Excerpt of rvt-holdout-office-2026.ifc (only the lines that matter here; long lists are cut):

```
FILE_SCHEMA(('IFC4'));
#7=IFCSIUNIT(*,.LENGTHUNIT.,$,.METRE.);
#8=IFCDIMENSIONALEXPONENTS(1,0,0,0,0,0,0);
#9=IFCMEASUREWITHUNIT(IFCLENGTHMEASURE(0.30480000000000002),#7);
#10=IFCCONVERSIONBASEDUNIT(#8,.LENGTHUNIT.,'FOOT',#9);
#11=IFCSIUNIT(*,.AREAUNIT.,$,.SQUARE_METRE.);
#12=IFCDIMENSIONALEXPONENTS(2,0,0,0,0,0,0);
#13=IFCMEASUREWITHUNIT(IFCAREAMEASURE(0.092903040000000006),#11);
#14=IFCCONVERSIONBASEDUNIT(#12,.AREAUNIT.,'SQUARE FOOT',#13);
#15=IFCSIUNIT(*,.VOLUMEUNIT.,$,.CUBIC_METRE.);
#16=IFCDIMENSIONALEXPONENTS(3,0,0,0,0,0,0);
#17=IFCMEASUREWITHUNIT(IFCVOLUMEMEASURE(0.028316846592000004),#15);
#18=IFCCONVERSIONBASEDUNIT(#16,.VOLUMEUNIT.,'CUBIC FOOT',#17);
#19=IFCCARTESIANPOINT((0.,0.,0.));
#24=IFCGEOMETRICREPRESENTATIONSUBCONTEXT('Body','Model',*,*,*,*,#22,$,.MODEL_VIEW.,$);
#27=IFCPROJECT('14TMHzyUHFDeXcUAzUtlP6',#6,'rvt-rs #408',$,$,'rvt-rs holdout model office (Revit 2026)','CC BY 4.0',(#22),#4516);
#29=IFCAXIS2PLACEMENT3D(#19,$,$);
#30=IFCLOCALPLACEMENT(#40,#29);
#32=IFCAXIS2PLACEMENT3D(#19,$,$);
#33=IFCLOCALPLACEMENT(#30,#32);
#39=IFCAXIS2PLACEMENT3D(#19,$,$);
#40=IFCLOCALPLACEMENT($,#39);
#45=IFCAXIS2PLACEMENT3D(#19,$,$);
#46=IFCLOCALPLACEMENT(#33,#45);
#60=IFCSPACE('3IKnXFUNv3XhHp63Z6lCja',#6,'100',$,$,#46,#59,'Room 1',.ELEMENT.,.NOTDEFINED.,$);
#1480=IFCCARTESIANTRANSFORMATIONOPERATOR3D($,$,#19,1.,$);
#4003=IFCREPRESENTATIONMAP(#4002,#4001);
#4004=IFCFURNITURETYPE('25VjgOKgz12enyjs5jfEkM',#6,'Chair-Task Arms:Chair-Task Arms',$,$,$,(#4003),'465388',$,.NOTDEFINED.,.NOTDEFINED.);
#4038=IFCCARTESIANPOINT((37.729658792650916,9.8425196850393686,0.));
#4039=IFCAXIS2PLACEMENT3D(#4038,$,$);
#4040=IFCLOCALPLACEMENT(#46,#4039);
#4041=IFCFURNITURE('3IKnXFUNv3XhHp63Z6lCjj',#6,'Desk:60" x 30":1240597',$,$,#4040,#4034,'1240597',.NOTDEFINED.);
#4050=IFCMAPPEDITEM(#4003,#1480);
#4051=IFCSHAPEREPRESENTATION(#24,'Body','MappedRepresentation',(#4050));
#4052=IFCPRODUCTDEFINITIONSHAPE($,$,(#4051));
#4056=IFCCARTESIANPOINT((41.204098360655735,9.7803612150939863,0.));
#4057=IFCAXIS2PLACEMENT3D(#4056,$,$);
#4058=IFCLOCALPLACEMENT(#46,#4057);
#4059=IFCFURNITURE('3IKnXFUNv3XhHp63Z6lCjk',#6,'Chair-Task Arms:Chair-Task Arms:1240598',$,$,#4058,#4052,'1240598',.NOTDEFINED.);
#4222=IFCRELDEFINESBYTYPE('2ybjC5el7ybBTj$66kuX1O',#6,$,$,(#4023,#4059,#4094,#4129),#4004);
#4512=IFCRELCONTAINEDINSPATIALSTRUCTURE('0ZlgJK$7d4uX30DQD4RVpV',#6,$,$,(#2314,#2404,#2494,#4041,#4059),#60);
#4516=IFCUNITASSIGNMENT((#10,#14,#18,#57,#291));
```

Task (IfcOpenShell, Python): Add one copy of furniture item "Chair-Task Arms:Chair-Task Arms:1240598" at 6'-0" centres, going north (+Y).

```python
import numpy as np
import ifcopenshell
import ifcopenshell.api.geometry
import ifcopenshell.api.root
import ifcopenshell.util.element
import ifcopenshell.util.placement
import ifcopenshell.util.unit

model = ifcopenshell.open("rvt-holdout-office-2026.ifc")
unit_scale = ifcopenshell.util.unit.calculate_unit_scale(model)


def reuse_history(source, copy):
    """copy_class also copies each property set's owner history, people and application; keep the originals."""
    for rel in copy.IsDefinedBy:
        if rel.is_a("IfcRelDefinesByProperties") and (history := rel.RelatingPropertyDefinition.OwnerHistory):
            rel.RelatingPropertyDefinition.OwnerHistory = source.OwnerHistory
            ifcopenshell.util.element.remove_deep2(model, history)


source = model.by_guid("3IKnXFUNv3XhHp63Z6lCjk")
base = ifcopenshell.util.placement.get_local_placement(source.ObjectPlacement)
step = np.array([0.0, 1.0, 0.0]) * 72 * 0.0254 / unit_scale

for i in range(1, 2):
    copy = ifcopenshell.api.root.copy_class(model, product=source)
    copy.Representation = ifcopenshell.util.element.copy_deep(
        model, source.Representation, exclude=["IfcGeometricRepresentationContext", "IfcRepresentationMap"]
    )
    copy.Name = "Chair-Task Arms:Chair-Task Arms"
    copy.Tag = None
    reuse_history(source, copy)
    matrix = base.copy()
    matrix[:3, 3] += i * step
    print("added at", matrix[:3, 3].round(3) + 0.0)
    ifcopenshell.api.geometry.edit_object_placement(model, product=copy, matrix=matrix, is_si=False)

model.write("rvt-holdout-office-2026_rev.ifc")
```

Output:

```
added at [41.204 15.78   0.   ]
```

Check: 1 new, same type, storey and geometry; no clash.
